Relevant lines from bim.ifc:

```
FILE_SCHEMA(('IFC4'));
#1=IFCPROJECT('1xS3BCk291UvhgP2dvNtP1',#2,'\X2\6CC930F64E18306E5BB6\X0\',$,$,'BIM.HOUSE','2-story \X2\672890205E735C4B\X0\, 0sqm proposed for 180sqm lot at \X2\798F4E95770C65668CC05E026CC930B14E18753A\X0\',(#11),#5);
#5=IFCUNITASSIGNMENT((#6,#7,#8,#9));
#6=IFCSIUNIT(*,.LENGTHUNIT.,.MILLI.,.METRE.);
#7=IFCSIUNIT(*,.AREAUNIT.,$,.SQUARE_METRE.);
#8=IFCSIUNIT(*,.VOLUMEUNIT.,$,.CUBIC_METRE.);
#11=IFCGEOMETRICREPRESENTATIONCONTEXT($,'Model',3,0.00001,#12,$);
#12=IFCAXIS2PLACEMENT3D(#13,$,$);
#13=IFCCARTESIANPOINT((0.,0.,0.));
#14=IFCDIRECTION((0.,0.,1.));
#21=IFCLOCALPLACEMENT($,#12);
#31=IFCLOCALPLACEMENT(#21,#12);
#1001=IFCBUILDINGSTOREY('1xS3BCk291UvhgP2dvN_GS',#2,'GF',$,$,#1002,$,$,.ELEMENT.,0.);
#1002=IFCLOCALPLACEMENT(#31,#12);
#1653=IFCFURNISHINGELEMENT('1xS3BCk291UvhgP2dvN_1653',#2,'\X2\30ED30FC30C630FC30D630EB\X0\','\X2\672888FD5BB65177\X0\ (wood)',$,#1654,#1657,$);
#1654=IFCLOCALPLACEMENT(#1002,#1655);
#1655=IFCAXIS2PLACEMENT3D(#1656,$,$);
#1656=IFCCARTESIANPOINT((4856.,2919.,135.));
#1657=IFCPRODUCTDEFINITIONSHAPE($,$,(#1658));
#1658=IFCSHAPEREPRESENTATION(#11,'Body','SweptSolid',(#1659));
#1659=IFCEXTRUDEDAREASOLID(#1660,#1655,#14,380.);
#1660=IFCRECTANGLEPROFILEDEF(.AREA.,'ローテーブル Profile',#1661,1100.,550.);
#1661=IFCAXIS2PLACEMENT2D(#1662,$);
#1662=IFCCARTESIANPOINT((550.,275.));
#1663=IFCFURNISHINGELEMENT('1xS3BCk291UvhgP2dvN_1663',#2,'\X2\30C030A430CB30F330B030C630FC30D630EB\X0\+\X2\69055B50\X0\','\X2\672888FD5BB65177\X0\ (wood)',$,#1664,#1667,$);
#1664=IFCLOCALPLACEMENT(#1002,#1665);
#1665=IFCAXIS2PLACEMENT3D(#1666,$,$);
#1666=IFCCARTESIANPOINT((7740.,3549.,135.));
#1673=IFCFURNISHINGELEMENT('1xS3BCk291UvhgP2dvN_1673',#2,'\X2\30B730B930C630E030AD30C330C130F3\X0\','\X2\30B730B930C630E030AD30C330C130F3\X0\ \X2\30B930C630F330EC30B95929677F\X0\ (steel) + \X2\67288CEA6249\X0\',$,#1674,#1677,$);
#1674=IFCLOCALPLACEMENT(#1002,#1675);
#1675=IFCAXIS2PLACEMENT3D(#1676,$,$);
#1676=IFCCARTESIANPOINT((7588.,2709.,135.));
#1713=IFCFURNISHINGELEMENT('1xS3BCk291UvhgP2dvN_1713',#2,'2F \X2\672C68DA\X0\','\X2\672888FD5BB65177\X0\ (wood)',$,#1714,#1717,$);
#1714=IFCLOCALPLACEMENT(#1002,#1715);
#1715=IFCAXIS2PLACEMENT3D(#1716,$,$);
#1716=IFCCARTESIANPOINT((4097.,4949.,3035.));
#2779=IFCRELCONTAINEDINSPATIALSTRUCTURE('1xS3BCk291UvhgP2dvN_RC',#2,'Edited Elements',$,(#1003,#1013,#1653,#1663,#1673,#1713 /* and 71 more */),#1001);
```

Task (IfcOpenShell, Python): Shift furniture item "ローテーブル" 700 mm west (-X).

```python
import ifcopenshell
import ifcopenshell.api.geometry
import ifcopenshell.util.placement

model = ifcopenshell.open("bim.ifc")

item = model.by_guid("1xS3BCk291UvhgP2dvN_1653")
matrix = ifcopenshell.util.placement.get_local_placement(item.ObjectPlacement)
matrix[0, 3] -= 700.0
ifcopenshell.api.geometry.edit_object_placement(model, product=item, matrix=matrix, is_si=False)

print(ifcopenshell.util.placement.get_local_placement(item.ObjectPlacement).round(3) + 0.0)

model.write("bim-out.ifc")
```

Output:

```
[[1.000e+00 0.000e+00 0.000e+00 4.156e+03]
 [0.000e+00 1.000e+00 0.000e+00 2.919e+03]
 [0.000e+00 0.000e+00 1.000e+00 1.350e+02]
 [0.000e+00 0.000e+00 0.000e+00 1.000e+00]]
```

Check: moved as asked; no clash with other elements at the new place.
